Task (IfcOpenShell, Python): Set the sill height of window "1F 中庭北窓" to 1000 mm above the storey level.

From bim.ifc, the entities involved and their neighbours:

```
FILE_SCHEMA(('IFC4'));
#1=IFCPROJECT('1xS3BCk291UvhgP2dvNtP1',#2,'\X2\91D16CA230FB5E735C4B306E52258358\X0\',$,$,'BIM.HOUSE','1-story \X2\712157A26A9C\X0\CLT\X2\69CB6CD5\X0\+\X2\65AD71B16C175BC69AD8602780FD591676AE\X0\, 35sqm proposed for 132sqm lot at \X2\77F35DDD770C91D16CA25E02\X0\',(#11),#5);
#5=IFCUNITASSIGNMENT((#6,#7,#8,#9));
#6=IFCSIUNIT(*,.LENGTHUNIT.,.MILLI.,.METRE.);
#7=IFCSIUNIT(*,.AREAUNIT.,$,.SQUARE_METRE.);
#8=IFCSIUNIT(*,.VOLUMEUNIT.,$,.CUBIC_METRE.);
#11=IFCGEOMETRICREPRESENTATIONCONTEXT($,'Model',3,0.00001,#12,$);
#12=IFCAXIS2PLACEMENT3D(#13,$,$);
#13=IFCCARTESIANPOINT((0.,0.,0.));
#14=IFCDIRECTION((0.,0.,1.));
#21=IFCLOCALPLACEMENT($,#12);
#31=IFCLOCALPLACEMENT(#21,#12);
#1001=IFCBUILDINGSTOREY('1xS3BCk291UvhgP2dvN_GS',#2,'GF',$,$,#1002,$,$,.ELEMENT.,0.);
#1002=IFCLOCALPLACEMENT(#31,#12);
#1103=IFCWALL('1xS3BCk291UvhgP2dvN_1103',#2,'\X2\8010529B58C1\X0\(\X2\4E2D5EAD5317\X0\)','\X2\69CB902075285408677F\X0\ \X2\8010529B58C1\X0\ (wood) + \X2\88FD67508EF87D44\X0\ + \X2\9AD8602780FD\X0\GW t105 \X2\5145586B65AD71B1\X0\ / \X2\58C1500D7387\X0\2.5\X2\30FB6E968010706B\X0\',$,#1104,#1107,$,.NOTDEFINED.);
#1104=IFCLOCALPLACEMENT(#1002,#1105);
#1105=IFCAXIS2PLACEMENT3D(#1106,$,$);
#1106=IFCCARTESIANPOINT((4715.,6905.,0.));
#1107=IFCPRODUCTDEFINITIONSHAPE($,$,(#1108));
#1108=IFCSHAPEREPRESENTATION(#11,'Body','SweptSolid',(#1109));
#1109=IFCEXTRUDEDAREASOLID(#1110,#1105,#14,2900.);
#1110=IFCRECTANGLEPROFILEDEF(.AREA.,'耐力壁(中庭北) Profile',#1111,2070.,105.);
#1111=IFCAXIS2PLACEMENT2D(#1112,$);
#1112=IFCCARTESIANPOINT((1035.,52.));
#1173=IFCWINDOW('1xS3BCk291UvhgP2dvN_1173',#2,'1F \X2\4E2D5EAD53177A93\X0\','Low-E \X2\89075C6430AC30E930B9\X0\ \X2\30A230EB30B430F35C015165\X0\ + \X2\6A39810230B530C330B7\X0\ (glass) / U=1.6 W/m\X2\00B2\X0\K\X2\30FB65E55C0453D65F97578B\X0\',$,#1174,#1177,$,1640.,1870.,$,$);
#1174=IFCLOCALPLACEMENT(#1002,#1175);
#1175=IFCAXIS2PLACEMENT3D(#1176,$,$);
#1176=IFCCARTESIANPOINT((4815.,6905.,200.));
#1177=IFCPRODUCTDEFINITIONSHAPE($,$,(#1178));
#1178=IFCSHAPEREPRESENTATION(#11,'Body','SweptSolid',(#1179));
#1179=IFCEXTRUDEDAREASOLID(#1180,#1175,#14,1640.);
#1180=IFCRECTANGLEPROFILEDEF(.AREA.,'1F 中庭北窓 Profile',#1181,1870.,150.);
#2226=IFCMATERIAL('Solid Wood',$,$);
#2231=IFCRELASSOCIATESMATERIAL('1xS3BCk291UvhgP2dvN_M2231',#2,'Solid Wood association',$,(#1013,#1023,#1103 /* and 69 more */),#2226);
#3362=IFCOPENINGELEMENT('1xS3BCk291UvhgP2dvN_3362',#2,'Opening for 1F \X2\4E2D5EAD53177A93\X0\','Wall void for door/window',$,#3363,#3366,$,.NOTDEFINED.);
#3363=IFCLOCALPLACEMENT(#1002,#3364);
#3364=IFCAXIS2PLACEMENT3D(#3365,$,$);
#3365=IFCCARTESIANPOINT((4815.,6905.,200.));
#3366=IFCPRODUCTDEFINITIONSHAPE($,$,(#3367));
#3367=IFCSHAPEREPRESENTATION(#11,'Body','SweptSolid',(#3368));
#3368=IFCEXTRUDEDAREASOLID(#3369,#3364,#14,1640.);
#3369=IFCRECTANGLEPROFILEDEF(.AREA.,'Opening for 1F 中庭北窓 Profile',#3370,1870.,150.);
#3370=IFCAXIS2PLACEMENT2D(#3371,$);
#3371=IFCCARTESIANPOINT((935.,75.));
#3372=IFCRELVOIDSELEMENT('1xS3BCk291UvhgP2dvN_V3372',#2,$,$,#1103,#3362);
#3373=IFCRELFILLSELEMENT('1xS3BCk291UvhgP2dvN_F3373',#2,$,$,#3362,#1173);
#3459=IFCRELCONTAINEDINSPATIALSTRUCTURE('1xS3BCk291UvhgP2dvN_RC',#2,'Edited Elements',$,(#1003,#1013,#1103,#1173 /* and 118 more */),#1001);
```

```python
import numpy as np
import ifcopenshell
import ifcopenshell.api.geometry
import ifcopenshell.geom
import ifcopenshell.util.element
import ifcopenshell.util.placement
import ifcopenshell.util.shape
import ifcopenshell.util.unit

model = ifcopenshell.open("bim.ifc")
unit_scale = ifcopenshell.util.unit.calculate_unit_scale(model)

window = model.by_guid("1xS3BCk291UvhgP2dvN_1173")
opening = window.FillsVoids[0].RelatingOpeningElement
storey = ifcopenshell.util.element.get_container(window, ifc_class="IfcBuildingStorey")
level = ifcopenshell.util.placement.get_local_placement(storey.ObjectPlacement)[2, 3]

# The opening's origin need not be at the sill, so measure its lowest point.
shape = ifcopenshell.geom.create_shape(ifcopenshell.geom.settings(), opening)
bottom = ifcopenshell.util.shape.get_shape_bottom_elevation(shape, shape.geometry) / unit_scale
dz = level + 1 / unit_scale - bottom

shift = np.array([0.0, 0.0, dz])
# The window is not placed relative to its opening, so move both.
for product in (opening, window):
    matrix = ifcopenshell.util.placement.get_local_placement(product.ObjectPlacement)
    matrix[:3, 3] += shift
    ifcopenshell.api.geometry.edit_object_placement(model, product=product, matrix=matrix, is_si=False)

print(f"moved by {dz * unit_scale:+.3f} m")

model.write("bim_v2.ifc")
```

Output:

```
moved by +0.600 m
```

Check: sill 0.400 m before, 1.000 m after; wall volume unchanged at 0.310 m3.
